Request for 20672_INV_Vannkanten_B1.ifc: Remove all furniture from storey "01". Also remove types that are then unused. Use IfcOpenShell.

First a look at what the model holds.

```python
import ifcopenshell
import ifcopenshell.util.element

model = ifcopenshell.open("20672_INV_Vannkanten_B1.ifc")
print(model.schema)
storey = next(s for s in model.by_type("IfcBuildingStorey") if s.Name == "01")
furniture = [e for e in ifcopenshell.util.element.get_decomposition(storey) if e.is_a("IfcFurnishingElement")]
seen = {}
for e in furniture:
    element_type = ifcopenshell.util.element.get_type(e)
    name = element_type.Name if element_type not in (None, e) else None
    seen[name] = seen.get(name, 0) + 1
for name, count in sorted(seen.items(), key=str):
    print(count, "x", name)
```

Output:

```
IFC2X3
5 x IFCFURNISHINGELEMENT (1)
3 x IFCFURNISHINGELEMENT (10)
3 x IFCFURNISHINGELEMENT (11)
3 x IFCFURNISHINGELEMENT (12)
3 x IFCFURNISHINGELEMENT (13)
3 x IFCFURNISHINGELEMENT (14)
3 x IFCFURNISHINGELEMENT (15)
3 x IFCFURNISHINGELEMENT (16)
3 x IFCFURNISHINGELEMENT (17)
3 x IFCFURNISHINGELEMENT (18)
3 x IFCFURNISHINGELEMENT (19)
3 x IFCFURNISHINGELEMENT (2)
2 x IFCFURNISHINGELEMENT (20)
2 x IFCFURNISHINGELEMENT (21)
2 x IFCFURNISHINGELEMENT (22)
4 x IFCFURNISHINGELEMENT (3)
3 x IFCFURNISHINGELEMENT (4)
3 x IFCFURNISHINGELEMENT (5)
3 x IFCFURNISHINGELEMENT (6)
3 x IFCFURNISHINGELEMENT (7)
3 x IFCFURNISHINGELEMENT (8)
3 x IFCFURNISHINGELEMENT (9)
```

```python
import ifcopenshell
import ifcopenshell.api.root
import ifcopenshell.util.element

model = ifcopenshell.open("20672_INV_Vannkanten_B1.ifc")

storey = next(s for s in model.by_type("IfcBuildingStorey") if s.Name == "01")
furniture = [e for e in ifcopenshell.util.element.get_decomposition(storey) if e.is_a("IfcFurnishingElement")]
types = {ifcopenshell.util.element.get_type(e) for e in furniture} - {None, *furniture}

for e in furniture:
    ifcopenshell.api.root.remove_product(model, product=e)
print(len(furniture), "removed")

unused = [t for t in types if not ifcopenshell.util.element.get_types(t)]
for t in unused:
    ifcopenshell.api.root.remove_product(model, product=t)
print(len(unused), "unused types removed")

model.write("20672_INV_Vannkanten_B1_rev.ifc")
```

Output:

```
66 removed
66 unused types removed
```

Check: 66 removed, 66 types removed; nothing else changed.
